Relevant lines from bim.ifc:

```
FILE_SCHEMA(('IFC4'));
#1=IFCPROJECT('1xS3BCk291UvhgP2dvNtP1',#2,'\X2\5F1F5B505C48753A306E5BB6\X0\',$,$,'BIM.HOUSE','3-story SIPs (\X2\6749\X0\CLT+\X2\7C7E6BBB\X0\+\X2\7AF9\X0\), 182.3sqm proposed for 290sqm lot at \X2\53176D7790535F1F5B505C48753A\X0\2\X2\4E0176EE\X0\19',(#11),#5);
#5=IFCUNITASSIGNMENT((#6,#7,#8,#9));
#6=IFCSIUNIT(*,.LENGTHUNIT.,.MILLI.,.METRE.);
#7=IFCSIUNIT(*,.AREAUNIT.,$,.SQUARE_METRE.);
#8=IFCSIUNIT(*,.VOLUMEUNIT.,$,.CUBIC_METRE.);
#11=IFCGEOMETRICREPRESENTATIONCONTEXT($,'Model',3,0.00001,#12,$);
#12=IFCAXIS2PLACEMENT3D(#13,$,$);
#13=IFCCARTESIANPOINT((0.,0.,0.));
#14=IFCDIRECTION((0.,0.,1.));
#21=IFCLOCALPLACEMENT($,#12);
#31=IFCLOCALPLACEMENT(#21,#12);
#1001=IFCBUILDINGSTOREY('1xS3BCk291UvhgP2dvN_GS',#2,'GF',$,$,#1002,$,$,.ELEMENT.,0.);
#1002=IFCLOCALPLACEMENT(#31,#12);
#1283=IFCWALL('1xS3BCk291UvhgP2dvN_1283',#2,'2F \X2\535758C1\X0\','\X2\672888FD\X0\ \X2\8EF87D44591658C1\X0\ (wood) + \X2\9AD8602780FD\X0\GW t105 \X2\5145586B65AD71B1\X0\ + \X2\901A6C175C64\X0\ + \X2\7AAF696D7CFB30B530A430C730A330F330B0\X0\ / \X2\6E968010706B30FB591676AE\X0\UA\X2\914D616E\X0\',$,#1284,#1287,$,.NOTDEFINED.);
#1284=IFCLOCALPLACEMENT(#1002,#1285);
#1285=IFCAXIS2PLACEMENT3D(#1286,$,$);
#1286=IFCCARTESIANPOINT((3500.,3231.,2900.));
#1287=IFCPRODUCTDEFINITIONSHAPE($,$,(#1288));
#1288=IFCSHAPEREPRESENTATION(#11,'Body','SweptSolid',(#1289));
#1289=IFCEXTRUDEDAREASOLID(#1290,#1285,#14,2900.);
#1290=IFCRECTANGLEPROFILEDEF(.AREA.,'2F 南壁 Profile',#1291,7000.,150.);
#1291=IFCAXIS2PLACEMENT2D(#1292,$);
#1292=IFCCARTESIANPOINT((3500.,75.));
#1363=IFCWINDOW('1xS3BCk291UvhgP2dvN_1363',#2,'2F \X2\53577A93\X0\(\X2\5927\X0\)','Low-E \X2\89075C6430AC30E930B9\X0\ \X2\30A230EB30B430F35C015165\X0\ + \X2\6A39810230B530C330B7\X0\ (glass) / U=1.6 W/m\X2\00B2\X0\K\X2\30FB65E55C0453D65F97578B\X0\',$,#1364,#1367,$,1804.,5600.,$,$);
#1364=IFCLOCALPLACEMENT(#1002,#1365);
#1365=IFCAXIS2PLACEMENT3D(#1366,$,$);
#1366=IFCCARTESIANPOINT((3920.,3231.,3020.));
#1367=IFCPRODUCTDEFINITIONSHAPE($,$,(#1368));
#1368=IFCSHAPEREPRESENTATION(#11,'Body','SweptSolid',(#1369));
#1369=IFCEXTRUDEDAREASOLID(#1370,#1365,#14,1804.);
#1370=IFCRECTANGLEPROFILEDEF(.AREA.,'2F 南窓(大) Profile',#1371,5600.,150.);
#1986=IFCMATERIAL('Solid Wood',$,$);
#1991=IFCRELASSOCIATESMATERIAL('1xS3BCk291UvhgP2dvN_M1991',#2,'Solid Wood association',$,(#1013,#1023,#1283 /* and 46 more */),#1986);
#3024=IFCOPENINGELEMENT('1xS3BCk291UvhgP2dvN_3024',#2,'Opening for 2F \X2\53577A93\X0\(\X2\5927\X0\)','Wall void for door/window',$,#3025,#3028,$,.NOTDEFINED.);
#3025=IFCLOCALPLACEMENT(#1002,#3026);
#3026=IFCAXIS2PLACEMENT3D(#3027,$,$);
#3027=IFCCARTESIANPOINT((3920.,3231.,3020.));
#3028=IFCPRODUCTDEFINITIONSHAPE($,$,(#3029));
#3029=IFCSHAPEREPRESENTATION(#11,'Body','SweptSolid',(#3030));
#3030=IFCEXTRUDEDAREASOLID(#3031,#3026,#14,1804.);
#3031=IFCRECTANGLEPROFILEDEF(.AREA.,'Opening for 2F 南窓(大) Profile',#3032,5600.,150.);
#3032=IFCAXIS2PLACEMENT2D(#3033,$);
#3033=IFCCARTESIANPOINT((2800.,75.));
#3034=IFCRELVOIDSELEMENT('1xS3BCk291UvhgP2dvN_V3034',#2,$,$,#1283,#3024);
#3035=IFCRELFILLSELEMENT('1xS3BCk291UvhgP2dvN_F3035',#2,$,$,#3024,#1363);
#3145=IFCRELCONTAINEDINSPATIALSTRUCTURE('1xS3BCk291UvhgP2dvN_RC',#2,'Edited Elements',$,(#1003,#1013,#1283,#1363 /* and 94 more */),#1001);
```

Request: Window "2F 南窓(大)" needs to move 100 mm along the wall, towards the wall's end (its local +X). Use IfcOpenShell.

```python
import ifcopenshell
import ifcopenshell.api.geometry
import ifcopenshell.util.placement
import ifcopenshell.util.unit

model = ifcopenshell.open("bim.ifc")
unit_scale = ifcopenshell.util.unit.calculate_unit_scale(model)

window = model.by_guid("1xS3BCk291UvhgP2dvN_1363")
opening = window.FillsVoids[0].RelatingOpeningElement
wall = opening.VoidsElements[0].RelatingBuildingElement

wall_matrix = ifcopenshell.util.placement.get_local_placement(wall.ObjectPlacement)
shift = wall_matrix[:3, 0] * 0.1 / unit_scale
before = ifcopenshell.util.placement.get_local_placement(window.ObjectPlacement)[:3, 3].copy()

# The window is not placed relative to its opening, so move both.
for product in (opening, window):
    matrix = ifcopenshell.util.placement.get_local_placement(product.ObjectPlacement)
    matrix[:3, 3] += shift
    ifcopenshell.api.geometry.edit_object_placement(model, product=product, matrix=matrix, is_si=False)

after = ifcopenshell.util.placement.get_local_placement(window.ObjectPlacement)[:3, 3]
print("window moved by", (after - before).round(3) + 0.0)

model.write("bim-out.ifc")
```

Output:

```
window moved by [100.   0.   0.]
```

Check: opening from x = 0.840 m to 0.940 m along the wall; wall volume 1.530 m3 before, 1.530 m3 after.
